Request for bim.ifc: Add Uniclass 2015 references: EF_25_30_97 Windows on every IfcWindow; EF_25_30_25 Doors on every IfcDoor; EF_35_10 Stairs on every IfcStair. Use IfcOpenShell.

First a look at what the model holds.

```python
import ifcopenshell

model = ifcopenshell.open("bim.ifc")
print(model.schema)
print("classifications:", [c.Name for c in model.by_type("IfcClassification")])
for ifc_class in ("IfcDoor", "IfcRoof", "IfcStair", "IfcWall", "IfcWindow"):
    print(ifc_class, len(model.by_type(ifc_class)))
```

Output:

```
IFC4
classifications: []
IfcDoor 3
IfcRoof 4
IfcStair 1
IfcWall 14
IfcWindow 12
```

```python
import ifcopenshell
import ifcopenshell.api.classification

model = ifcopenshell.open("bim.ifc")

system = ifcopenshell.api.classification.add_classification(model, classification="Uniclass 2015")

codes = {
    "IfcWindow": ("EF_25_30_97", "Windows"),
    "IfcDoor": ("EF_25_30_25", "Doors"),
    "IfcStair": ("EF_35_10", "Stairs"),
}
for ifc_class, (code, name) in codes.items():
    products = model.by_type(ifc_class)
    ifcopenshell.api.classification.add_reference(
        model, products=products, classification=system, identification=code, name=name
    )
    print(code, len(products))

model.write("bim_edited.ifc")
```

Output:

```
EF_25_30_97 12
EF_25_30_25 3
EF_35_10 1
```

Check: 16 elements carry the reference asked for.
